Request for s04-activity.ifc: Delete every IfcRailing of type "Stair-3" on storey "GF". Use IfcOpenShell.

First a look at what the model holds.

```python
import ifcopenshell
import ifcopenshell.util.element

model = ifcopenshell.open("s04-activity.ifc")
print(model.schema)
storey = next(s for s in model.by_type("IfcBuildingStorey") if s.Name == "GF")
railings = [e for e in ifcopenshell.util.element.get_decomposition(storey) if e.is_a("IfcRailing")]
seen = {}
for e in railings:
    element_type = ifcopenshell.util.element.get_type(e)
    name = element_type.Name if element_type not in (None, e) else None
    seen[name] = seen.get(name, 0) + 1
for name, count in sorted(seen.items(), key=str):
    print(count, "x", name)
```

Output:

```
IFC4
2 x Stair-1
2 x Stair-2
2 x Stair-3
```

```python
import ifcopenshell
import ifcopenshell.api.root
import ifcopenshell.util.element

model = ifcopenshell.open("s04-activity.ifc")

storey = next(s for s in model.by_type("IfcBuildingStorey") if s.Name == "GF")
railings = [e for e in ifcopenshell.util.element.get_decomposition(storey) if e.is_a("IfcRailing")]
targets = [e for e in railings if (t := ifcopenshell.util.element.get_type(e)) not in (None, e) and t.Name == "Stair-3"]

for e in targets:
    ifcopenshell.api.root.remove_product(model, product=e)
print(len(targets), "removed")

model.write("s04-activity_rev.ifc")
```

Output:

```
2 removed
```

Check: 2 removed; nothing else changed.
